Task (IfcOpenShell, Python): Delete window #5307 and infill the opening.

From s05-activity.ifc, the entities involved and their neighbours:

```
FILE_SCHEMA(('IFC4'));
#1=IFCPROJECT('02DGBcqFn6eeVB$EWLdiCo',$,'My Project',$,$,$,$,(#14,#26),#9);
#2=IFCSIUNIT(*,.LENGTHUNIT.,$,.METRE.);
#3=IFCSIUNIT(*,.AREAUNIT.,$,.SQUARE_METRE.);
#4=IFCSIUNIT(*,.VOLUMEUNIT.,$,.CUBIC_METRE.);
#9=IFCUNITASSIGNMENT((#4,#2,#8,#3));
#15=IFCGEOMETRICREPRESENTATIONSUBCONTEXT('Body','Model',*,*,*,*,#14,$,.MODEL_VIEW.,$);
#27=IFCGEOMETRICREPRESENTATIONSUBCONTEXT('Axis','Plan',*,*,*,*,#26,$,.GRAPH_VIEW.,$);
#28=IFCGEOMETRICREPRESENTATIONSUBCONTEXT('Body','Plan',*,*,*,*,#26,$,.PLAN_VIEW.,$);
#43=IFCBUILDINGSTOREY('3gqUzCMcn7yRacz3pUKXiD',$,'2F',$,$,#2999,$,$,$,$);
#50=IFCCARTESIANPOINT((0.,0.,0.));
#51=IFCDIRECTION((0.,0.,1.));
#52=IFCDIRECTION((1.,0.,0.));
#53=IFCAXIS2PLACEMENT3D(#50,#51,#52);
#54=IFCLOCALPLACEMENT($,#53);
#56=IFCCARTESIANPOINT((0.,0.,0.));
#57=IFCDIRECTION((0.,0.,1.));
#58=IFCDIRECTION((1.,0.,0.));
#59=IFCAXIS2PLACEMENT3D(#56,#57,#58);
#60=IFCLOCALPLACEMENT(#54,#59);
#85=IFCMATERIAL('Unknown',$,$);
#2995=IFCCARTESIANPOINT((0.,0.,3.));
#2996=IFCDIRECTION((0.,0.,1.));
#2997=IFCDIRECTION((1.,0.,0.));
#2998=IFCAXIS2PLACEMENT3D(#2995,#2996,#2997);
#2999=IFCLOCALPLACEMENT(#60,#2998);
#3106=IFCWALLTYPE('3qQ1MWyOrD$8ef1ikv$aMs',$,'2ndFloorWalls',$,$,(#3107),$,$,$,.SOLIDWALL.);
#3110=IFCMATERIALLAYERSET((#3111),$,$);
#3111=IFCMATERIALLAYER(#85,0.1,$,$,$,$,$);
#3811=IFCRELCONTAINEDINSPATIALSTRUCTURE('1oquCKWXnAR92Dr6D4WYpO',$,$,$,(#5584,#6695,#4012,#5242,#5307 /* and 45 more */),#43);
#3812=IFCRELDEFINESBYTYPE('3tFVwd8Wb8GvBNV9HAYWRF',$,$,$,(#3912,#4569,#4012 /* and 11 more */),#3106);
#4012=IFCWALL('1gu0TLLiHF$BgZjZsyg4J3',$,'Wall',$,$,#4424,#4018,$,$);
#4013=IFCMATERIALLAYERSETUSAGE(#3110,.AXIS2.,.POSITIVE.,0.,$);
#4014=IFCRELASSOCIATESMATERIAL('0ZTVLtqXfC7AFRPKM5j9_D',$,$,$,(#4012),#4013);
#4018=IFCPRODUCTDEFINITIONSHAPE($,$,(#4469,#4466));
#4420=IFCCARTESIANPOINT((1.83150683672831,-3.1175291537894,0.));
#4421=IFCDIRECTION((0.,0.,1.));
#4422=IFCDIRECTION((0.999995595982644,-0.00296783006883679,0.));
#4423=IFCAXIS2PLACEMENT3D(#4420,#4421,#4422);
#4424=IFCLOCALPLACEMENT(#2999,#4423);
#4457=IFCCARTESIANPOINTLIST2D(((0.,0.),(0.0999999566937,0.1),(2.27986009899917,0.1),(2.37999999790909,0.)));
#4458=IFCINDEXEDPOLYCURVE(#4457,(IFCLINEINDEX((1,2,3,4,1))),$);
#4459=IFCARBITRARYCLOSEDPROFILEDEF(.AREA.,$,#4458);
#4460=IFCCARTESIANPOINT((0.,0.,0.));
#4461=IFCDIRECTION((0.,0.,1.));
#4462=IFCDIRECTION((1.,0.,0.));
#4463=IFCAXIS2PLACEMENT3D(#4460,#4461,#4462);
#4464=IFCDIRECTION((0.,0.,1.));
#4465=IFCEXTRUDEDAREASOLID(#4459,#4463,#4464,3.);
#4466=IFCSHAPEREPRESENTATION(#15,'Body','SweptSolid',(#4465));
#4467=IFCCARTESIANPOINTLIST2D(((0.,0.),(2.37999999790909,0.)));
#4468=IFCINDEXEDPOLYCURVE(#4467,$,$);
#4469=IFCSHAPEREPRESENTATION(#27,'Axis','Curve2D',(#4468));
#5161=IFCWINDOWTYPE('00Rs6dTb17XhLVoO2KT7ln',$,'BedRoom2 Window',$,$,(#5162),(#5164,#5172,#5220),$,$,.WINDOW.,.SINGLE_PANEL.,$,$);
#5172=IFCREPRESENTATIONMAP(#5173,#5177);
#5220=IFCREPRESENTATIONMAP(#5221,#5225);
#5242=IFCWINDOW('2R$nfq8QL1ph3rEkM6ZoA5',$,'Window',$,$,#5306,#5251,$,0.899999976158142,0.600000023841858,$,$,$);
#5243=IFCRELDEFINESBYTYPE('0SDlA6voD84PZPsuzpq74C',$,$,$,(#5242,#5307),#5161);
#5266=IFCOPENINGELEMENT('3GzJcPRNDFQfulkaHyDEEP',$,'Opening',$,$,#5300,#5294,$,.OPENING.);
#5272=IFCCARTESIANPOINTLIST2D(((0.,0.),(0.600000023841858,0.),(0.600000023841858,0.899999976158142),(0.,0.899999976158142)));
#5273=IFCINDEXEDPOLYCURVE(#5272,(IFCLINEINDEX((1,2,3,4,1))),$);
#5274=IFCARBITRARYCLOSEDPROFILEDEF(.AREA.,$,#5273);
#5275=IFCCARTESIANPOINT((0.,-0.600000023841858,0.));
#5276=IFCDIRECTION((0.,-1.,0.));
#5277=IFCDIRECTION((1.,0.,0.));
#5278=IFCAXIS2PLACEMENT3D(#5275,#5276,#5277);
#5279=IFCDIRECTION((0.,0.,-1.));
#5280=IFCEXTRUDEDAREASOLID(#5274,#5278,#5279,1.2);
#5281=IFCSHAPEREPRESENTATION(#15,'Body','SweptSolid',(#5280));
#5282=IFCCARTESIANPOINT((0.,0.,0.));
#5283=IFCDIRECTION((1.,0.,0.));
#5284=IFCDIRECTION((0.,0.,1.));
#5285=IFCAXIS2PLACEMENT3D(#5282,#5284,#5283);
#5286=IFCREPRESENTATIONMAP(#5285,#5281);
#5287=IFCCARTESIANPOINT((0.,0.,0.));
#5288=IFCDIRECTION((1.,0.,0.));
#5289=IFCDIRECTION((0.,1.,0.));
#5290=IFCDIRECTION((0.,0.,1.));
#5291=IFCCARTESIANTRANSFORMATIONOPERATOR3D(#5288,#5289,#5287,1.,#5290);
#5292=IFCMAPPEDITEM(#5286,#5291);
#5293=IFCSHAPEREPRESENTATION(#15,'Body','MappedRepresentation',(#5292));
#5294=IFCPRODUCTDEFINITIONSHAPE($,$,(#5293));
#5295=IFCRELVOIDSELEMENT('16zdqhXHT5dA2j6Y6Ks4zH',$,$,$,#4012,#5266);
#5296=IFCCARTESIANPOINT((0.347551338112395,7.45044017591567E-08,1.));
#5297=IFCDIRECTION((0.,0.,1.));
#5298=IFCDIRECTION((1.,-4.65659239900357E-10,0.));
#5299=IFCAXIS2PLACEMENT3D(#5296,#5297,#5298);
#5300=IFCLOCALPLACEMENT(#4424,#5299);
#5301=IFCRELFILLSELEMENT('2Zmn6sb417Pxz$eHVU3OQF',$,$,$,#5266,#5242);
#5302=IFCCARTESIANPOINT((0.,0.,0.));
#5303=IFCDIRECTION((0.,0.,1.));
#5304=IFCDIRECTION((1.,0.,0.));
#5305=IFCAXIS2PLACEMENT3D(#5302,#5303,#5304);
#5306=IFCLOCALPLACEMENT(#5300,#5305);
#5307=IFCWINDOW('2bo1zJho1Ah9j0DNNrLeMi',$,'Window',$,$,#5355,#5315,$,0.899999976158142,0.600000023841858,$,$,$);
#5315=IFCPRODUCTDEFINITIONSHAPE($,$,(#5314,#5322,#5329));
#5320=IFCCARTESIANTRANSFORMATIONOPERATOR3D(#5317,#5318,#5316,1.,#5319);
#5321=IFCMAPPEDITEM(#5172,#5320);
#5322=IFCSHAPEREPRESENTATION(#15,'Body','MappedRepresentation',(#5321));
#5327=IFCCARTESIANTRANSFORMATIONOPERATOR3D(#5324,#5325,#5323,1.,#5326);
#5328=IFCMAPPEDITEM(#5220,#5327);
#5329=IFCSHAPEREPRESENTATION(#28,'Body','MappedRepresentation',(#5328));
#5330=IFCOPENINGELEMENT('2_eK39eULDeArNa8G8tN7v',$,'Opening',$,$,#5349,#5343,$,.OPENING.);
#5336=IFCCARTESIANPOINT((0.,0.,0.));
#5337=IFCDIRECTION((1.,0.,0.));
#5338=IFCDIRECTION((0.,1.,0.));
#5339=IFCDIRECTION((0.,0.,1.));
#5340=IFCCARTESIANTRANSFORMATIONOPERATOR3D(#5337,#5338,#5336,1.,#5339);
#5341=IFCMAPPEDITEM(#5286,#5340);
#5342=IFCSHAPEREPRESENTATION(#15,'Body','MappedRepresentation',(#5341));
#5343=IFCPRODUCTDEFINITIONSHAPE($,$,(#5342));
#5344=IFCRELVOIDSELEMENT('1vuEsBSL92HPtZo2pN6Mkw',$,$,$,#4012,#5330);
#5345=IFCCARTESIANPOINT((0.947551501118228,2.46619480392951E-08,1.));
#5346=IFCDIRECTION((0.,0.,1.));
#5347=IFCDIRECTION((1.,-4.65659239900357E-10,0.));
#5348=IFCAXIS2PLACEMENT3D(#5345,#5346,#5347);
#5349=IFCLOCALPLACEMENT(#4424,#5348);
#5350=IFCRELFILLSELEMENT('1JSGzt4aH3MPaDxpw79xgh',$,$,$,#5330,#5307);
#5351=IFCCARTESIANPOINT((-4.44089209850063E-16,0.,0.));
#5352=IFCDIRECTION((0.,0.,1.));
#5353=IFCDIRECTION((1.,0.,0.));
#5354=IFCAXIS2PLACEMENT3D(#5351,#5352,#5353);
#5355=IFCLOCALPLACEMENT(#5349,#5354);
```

```python
import ifcopenshell
import ifcopenshell.api.feature
import ifcopenshell.api.root
import ifcopenshell.geom
import ifcopenshell.util.shape

model = ifcopenshell.open("s05-activity.ifc")
settings = ifcopenshell.geom.settings()


def volume(element):
    """Net volume in cubic metres, openings subtracted."""
    shape = ifcopenshell.geom.create_shape(settings, element)
    return ifcopenshell.util.shape.get_volume(shape.geometry)


window = model.by_id(5307)
opening = window.FillsVoids[0].RelatingOpeningElement
wall = opening.VoidsElements[0].RelatingBuildingElement
before = volume(wall)

ifcopenshell.api.root.remove_product(model, product=window)
ifcopenshell.api.feature.remove_feature(model, feature=opening)

after = volume(wall)

print(f"wall volume {before:.3f} -> {after:.3f} m3")

model.write("s05-activity_rev.ifc")
```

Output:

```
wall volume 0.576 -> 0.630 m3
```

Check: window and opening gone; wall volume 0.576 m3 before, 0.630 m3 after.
